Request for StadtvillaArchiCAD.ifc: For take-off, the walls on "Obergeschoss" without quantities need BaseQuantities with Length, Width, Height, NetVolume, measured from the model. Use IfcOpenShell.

First a look at what the model holds.

```python
import ifcopenshell
import ifcopenshell.util.element
import ifcopenshell.util.unit

model = ifcopenshell.open("StadtvillaArchiCAD.ifc")
print(model.schema)
for unit_type in ("LENGTHUNIT", "AREAUNIT", "VOLUMEUNIT"):
    print(unit_type, ifcopenshell.util.unit.calculate_unit_scale(model, unit_type))
storey = next(s for s in model.by_type("IfcBuildingStorey") if s.Name == "Obergeschoss")
walls = [e for e in ifcopenshell.util.element.get_decomposition(storey) if e.is_a("IfcWall")]
for e in sorted(walls, key=lambda e: e.id()):
    print(e.id(), e.is_a(), e.Name, list(ifcopenshell.util.element.get_psets(e, qtos_only=True)), sep=" | ")
```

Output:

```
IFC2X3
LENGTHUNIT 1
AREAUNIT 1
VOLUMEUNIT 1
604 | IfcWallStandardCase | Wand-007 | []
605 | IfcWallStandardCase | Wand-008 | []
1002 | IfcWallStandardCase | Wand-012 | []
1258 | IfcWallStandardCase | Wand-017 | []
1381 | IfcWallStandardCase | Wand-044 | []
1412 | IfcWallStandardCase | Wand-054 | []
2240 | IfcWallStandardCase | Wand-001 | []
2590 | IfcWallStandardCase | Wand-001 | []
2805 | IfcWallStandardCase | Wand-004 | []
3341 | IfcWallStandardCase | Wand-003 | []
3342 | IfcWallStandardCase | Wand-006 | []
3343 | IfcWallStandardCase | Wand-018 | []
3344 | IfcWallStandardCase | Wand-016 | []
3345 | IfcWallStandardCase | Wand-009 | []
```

```python
import ifcopenshell
import ifcopenshell.api.pset
import ifcopenshell.geom
import ifcopenshell.util.element
import ifcopenshell.util.shape
import ifcopenshell.util.unit

model = ifcopenshell.open("StadtvillaArchiCAD.ifc")
unit_scale = ifcopenshell.util.unit.calculate_unit_scale(model)
volume_scale = ifcopenshell.util.unit.calculate_unit_scale(model, "VOLUMEUNIT")
settings = ifcopenshell.geom.settings()

storey = next(s for s in model.by_type("IfcBuildingStorey") if s.Name == "Obergeschoss")
walls = [e for e in ifcopenshell.util.element.get_decomposition(storey) if e.is_a("IfcWall")]

for e in sorted(walls, key=lambda e: e.id()):
    if ifcopenshell.util.element.get_psets(e, qtos_only=True, should_inherit=False):
        continue
    # Geometry comes back in metres, in the element's own axes.
    shape = ifcopenshell.geom.create_shape(settings, e)
    values = {
        "Length": ifcopenshell.util.shape.get_x(shape.geometry) / unit_scale,
        "Width": ifcopenshell.util.shape.get_y(shape.geometry) / unit_scale,
        "Height": ifcopenshell.util.shape.get_z(shape.geometry) / unit_scale,
        "NetVolume": ifcopenshell.util.shape.get_volume(shape.geometry) / volume_scale,
    }
    qto = ifcopenshell.api.pset.add_qto(model, product=e, name="BaseQuantities")
    ifcopenshell.api.pset.edit_qto(model, qto=qto, properties=values)
    print(e.id(), {k: round(v, 3) for k, v in values.items()})

model.write("StadtvillaArchiCAD-out.ifc")
```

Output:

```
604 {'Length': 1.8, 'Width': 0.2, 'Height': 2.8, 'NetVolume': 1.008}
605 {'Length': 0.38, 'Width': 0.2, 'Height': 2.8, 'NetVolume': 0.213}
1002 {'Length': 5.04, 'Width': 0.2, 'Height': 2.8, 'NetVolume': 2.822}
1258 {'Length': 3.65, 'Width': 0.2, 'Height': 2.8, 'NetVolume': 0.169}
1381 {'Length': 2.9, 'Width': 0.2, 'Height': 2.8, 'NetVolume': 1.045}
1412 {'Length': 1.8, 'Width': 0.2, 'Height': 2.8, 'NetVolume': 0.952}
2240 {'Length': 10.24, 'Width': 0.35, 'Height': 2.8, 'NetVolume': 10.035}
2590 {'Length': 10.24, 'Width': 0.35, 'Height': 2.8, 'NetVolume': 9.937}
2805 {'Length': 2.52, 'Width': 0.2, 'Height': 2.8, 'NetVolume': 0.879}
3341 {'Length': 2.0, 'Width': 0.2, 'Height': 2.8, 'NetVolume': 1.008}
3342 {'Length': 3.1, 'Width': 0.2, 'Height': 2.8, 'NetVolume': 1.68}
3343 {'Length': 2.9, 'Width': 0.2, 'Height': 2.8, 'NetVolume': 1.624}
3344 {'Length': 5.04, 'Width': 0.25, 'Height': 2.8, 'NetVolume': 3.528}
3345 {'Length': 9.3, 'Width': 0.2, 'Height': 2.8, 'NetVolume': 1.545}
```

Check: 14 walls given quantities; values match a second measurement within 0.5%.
